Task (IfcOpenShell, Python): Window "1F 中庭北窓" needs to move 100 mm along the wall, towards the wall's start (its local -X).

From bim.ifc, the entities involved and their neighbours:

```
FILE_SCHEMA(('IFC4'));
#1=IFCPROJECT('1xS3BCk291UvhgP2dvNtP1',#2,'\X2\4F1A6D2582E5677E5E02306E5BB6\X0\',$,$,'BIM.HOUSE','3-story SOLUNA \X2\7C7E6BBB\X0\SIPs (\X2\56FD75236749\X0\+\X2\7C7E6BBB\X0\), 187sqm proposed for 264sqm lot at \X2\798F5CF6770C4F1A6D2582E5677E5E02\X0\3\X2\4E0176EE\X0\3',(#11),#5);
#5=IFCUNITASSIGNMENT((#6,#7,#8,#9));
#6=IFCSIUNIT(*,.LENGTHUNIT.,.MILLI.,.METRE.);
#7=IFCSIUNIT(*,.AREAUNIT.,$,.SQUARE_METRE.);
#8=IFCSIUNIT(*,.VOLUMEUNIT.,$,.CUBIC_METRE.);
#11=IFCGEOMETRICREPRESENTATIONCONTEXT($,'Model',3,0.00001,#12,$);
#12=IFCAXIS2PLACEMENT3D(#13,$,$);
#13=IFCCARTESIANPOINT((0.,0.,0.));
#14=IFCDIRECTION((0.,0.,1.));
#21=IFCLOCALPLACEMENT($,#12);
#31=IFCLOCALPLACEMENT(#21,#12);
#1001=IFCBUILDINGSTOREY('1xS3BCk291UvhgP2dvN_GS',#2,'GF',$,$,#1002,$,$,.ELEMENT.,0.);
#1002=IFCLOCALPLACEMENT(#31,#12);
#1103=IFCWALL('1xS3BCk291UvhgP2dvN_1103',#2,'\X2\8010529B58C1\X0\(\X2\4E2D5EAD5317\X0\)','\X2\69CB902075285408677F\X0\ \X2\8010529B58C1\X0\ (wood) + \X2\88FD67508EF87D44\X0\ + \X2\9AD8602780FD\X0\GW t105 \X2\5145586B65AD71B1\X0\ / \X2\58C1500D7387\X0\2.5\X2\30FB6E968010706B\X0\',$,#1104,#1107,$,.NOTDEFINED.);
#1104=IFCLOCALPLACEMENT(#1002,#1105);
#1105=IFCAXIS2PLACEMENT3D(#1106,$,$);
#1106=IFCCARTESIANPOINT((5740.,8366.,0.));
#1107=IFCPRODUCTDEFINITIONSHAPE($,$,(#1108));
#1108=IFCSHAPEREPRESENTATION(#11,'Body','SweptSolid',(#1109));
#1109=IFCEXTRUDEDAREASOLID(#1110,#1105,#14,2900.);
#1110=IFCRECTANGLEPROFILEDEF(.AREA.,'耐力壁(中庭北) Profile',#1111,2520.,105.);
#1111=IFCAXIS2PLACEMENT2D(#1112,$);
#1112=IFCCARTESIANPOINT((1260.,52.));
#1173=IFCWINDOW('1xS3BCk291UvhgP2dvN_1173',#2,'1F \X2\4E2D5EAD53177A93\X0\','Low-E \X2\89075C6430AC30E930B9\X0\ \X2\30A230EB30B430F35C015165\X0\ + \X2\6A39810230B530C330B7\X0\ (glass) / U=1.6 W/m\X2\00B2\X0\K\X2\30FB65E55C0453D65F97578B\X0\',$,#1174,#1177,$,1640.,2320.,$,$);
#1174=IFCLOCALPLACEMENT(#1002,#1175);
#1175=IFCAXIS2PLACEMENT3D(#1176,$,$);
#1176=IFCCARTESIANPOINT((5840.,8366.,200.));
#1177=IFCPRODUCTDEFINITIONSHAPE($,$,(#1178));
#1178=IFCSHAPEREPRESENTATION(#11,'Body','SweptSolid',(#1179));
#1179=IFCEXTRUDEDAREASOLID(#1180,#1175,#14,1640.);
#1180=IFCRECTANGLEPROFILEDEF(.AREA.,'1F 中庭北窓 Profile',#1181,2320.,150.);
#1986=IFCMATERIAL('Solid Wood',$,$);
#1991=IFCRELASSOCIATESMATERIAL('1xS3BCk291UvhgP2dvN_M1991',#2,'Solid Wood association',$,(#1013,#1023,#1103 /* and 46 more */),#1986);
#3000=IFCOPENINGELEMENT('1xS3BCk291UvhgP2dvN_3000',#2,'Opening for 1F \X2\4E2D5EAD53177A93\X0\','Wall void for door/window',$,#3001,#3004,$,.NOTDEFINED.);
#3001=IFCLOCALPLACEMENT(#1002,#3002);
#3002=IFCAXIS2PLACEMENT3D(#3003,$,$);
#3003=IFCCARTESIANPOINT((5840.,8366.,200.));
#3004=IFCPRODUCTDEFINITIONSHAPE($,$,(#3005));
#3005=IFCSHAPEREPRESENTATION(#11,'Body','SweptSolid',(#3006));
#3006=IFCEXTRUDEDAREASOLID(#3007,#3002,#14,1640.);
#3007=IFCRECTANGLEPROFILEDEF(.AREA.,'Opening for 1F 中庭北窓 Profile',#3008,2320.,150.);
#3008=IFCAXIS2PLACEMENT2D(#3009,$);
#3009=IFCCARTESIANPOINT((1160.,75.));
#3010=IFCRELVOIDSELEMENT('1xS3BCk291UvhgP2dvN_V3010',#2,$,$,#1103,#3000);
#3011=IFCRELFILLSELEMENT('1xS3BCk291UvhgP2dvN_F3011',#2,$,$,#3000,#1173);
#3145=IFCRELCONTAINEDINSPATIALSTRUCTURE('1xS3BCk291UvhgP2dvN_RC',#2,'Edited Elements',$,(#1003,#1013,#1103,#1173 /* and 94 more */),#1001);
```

```python
import ifcopenshell
import ifcopenshell.api.geometry
import ifcopenshell.util.placement

model = ifcopenshell.open("bim.ifc")

window = model.by_guid("1xS3BCk291UvhgP2dvN_1173")
opening = window.FillsVoids[0].RelatingOpeningElement
wall = opening.VoidsElements[0].RelatingBuildingElement

wall_matrix = ifcopenshell.util.placement.get_local_placement(wall.ObjectPlacement)
shift = wall_matrix[:3, 0] * -100.0
before = ifcopenshell.util.placement.get_local_placement(window.ObjectPlacement)[:3, 3].copy()

# The window is not placed relative to its opening, so move both.
for product in (opening, window):
    matrix = ifcopenshell.util.placement.get_local_placement(product.ObjectPlacement)
    matrix[:3, 3] += shift
    ifcopenshell.api.geometry.edit_object_placement(model, product=product, matrix=matrix, is_si=False)

after = ifcopenshell.util.placement.get_local_placement(window.ObjectPlacement)[:3, 3]
print("window moved by", (after - before).round(3) + 0.0)

model.write("bim-out.ifc")
```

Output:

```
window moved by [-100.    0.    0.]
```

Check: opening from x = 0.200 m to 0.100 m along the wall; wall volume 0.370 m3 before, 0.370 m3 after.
